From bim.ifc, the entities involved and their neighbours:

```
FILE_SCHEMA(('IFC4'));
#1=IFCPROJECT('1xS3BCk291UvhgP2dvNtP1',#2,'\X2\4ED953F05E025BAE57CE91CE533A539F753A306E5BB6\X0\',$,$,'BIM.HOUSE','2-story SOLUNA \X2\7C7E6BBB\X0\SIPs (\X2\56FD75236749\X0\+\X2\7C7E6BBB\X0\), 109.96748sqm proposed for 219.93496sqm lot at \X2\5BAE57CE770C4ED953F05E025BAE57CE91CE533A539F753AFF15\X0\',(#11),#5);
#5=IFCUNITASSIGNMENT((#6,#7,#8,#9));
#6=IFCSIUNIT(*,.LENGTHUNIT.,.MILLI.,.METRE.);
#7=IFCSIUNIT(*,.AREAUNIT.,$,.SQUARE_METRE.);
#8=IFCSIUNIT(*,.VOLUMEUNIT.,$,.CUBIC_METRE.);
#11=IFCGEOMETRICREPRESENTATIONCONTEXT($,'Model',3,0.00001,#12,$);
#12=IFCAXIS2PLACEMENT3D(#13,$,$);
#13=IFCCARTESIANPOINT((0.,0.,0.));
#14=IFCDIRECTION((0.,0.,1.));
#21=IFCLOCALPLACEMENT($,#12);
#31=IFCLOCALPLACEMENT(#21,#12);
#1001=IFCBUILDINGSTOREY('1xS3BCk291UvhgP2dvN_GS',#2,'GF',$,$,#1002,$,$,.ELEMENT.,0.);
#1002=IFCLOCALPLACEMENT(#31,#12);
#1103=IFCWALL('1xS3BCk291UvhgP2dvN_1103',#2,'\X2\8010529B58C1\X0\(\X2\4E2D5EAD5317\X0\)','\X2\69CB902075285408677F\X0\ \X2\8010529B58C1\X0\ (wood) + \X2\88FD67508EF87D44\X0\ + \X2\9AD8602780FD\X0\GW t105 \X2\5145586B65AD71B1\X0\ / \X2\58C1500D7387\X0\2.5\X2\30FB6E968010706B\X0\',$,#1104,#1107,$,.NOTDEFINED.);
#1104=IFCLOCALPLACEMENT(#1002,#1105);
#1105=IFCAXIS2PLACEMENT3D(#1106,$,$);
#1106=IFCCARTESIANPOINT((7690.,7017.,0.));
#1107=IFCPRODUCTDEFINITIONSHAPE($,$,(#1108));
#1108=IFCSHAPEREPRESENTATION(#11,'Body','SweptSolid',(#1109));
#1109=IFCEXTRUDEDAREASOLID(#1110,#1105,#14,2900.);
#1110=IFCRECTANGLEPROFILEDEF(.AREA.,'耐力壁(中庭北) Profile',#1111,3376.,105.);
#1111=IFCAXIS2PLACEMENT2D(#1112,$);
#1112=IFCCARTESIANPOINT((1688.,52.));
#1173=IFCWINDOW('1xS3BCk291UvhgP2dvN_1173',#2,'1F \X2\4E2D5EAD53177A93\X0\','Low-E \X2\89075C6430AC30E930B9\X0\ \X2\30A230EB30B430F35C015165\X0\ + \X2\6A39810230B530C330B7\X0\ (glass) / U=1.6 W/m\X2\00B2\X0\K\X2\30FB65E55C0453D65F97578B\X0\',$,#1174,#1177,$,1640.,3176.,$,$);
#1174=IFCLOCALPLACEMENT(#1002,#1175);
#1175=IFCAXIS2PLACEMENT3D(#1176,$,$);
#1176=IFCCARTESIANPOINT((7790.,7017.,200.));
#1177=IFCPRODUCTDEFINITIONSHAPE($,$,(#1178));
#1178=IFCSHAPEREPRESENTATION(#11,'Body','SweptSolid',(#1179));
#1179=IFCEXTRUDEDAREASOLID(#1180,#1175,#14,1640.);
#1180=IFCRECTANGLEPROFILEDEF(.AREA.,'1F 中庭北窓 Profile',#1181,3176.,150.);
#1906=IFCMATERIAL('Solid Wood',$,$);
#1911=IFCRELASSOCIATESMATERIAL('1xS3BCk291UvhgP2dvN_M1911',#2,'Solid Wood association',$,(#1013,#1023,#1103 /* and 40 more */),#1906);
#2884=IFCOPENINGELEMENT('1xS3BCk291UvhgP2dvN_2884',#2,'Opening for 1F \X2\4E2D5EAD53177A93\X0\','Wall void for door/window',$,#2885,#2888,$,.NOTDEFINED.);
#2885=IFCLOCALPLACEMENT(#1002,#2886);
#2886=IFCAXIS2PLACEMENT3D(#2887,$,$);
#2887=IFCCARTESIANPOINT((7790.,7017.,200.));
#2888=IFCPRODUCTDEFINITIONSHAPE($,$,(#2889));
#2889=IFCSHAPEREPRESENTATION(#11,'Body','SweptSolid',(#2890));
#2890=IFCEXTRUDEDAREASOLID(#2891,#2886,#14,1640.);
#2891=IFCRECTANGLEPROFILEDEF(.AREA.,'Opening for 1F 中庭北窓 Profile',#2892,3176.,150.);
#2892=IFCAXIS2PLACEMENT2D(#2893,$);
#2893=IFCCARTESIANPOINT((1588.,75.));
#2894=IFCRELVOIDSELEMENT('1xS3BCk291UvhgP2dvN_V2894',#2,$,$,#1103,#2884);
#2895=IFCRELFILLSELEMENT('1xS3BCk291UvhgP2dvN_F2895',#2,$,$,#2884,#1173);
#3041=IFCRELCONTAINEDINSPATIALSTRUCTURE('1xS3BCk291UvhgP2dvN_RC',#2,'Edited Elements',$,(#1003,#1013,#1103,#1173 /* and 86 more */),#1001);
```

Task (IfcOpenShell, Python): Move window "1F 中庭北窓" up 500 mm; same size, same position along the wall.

```python
import numpy as np
import ifcopenshell
import ifcopenshell.api.geometry
import ifcopenshell.util.placement
import ifcopenshell.util.unit

model = ifcopenshell.open("bim.ifc")
unit_scale = ifcopenshell.util.unit.calculate_unit_scale(model)

window = model.by_guid("1xS3BCk291UvhgP2dvN_1173")
opening = window.FillsVoids[0].RelatingOpeningElement
dz = 0.5 / unit_scale

shift = np.array([0.0, 0.0, dz])
# The window is not placed relative to its opening, so move both.
for product in (opening, window):
    matrix = ifcopenshell.util.placement.get_local_placement(product.ObjectPlacement)
    matrix[:3, 3] += shift
    ifcopenshell.api.geometry.edit_object_placement(model, product=product, matrix=matrix, is_si=False)

print(f"moved by {dz * unit_scale:+.3f} m")

model.write("bim_v2.ifc")
```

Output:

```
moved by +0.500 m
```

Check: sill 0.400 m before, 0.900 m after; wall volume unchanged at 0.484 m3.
